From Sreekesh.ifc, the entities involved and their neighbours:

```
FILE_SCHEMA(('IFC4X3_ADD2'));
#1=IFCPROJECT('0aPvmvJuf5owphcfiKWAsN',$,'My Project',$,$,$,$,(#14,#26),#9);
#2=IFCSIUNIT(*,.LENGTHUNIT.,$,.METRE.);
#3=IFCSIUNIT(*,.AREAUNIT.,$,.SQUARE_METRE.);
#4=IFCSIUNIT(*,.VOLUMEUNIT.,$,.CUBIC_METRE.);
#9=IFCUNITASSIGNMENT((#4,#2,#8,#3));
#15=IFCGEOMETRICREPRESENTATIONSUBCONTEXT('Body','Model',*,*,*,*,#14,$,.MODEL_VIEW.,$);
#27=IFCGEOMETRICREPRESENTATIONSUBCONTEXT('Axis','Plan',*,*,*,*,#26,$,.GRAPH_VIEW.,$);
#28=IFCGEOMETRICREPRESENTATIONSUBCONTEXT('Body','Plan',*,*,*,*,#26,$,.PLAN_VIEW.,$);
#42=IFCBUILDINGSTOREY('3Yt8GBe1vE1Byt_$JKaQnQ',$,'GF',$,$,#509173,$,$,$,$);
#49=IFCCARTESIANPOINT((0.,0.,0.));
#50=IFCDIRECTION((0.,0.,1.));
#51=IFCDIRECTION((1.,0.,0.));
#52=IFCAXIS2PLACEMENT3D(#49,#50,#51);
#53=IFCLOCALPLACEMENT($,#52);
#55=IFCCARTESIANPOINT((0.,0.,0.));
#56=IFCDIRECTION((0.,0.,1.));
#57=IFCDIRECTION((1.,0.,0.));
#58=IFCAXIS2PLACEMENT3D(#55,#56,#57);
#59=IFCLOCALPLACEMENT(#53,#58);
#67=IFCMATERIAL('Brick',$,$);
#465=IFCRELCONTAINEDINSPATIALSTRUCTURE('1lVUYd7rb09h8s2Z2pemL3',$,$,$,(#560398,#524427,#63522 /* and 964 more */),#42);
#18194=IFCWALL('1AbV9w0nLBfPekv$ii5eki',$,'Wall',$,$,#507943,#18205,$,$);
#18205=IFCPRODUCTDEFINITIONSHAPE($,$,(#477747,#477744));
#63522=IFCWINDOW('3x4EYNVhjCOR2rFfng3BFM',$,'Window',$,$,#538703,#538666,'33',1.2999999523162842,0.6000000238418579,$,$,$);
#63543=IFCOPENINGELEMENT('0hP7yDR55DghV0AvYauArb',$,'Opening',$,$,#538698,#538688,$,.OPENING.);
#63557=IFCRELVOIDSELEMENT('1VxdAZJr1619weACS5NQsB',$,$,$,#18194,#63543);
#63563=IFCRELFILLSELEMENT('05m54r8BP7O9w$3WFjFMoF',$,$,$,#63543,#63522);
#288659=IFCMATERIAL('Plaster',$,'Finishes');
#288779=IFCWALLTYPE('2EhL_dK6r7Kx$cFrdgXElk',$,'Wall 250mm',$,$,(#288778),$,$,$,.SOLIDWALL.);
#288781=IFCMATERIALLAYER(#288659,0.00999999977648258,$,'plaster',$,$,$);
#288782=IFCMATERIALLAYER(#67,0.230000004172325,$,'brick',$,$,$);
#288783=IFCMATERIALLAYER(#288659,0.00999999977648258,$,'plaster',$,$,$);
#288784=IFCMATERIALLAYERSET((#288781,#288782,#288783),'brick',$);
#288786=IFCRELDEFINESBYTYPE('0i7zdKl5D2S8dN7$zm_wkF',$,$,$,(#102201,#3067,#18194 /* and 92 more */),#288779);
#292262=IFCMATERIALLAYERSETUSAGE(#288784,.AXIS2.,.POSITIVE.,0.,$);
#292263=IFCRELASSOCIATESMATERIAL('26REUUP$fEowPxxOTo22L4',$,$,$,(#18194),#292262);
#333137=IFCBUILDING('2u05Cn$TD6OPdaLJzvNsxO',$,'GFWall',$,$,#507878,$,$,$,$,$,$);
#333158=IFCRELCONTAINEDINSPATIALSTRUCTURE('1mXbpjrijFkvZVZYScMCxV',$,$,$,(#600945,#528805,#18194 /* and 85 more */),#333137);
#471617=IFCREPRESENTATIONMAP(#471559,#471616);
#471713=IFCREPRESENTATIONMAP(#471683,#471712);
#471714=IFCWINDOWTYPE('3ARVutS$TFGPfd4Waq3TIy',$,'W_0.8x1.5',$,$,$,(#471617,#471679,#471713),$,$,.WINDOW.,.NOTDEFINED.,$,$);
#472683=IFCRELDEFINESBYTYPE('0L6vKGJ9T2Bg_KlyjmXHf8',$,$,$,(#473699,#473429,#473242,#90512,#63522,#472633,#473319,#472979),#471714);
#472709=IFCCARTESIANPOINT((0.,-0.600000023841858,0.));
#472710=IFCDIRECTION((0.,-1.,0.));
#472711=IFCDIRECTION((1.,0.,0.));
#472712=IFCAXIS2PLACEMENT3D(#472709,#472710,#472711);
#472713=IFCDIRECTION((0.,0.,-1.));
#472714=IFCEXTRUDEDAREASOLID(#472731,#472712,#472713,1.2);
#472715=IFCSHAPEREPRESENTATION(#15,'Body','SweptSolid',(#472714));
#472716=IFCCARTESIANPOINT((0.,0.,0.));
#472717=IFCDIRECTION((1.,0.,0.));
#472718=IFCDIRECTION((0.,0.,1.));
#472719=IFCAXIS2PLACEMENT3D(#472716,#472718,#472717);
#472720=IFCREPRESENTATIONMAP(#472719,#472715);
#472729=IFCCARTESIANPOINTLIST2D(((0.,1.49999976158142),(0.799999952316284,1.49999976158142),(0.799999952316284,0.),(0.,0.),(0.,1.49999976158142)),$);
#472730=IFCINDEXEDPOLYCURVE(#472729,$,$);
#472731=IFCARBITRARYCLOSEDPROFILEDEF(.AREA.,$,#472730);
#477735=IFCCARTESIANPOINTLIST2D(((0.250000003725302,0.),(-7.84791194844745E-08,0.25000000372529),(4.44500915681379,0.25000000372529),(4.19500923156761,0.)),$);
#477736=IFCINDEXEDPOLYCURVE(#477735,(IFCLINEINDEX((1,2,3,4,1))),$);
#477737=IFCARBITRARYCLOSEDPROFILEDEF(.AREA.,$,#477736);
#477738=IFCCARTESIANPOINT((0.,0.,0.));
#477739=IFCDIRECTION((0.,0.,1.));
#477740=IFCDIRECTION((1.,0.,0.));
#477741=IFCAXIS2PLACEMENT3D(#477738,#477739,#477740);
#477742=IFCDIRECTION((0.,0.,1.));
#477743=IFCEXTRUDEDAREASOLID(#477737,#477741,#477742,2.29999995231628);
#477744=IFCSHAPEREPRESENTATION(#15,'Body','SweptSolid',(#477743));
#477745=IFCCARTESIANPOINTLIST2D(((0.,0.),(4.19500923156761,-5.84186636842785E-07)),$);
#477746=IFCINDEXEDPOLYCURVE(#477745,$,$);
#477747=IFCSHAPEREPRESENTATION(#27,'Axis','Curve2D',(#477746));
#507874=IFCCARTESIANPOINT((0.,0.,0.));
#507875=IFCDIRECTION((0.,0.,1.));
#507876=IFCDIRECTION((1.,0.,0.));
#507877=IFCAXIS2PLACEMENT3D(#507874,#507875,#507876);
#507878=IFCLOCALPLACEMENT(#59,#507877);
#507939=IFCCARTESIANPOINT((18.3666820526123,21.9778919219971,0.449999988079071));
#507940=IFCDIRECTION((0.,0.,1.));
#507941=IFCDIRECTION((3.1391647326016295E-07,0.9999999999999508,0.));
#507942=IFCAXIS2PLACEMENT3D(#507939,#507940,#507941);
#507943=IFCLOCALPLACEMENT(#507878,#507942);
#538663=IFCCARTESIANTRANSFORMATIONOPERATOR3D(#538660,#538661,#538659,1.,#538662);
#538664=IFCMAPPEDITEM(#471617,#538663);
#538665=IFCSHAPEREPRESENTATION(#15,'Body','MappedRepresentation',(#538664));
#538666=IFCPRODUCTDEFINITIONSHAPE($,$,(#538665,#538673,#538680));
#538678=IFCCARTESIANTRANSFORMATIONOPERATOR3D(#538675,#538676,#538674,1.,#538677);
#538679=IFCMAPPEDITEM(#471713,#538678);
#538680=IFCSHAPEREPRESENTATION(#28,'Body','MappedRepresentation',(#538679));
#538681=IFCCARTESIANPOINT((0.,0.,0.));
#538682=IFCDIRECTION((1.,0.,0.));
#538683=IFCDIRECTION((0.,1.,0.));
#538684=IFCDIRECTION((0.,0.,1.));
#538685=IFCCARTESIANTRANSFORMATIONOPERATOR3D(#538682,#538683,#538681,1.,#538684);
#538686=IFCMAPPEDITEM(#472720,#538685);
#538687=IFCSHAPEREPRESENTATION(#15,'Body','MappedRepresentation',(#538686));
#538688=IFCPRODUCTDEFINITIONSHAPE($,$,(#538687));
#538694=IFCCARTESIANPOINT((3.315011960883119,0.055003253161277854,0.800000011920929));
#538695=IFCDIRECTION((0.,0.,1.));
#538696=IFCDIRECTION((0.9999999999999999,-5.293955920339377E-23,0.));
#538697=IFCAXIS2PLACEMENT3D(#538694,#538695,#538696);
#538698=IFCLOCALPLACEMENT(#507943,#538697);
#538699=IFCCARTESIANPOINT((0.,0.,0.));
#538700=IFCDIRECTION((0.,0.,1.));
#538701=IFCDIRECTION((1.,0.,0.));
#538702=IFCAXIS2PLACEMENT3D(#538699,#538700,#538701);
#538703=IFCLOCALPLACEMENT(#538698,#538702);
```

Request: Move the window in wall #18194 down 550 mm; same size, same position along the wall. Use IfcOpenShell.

```python
import numpy as np
import ifcopenshell
import ifcopenshell.api.geometry
import ifcopenshell.util.placement
import ifcopenshell.util.unit

model = ifcopenshell.open("Sreekesh.ifc")
unit_scale = ifcopenshell.util.unit.calculate_unit_scale(model)

window = model.by_id(63522)
opening = window.FillsVoids[0].RelatingOpeningElement
dz = -0.55 / unit_scale

shift = np.array([0.0, 0.0, dz])
# The window is placed relative to its opening, so it follows when the opening moves.
matrix = ifcopenshell.util.placement.get_local_placement(opening.ObjectPlacement)
matrix[:3, 3] += shift
ifcopenshell.api.geometry.edit_object_placement(
    model, product=opening, matrix=matrix, is_si=False, should_transform_children=True
)

print(f"moved by {dz * unit_scale:+.3f} m")

model.write("Sreekesh_v2.ifc")
```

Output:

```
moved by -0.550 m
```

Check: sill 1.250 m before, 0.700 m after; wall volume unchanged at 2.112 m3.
